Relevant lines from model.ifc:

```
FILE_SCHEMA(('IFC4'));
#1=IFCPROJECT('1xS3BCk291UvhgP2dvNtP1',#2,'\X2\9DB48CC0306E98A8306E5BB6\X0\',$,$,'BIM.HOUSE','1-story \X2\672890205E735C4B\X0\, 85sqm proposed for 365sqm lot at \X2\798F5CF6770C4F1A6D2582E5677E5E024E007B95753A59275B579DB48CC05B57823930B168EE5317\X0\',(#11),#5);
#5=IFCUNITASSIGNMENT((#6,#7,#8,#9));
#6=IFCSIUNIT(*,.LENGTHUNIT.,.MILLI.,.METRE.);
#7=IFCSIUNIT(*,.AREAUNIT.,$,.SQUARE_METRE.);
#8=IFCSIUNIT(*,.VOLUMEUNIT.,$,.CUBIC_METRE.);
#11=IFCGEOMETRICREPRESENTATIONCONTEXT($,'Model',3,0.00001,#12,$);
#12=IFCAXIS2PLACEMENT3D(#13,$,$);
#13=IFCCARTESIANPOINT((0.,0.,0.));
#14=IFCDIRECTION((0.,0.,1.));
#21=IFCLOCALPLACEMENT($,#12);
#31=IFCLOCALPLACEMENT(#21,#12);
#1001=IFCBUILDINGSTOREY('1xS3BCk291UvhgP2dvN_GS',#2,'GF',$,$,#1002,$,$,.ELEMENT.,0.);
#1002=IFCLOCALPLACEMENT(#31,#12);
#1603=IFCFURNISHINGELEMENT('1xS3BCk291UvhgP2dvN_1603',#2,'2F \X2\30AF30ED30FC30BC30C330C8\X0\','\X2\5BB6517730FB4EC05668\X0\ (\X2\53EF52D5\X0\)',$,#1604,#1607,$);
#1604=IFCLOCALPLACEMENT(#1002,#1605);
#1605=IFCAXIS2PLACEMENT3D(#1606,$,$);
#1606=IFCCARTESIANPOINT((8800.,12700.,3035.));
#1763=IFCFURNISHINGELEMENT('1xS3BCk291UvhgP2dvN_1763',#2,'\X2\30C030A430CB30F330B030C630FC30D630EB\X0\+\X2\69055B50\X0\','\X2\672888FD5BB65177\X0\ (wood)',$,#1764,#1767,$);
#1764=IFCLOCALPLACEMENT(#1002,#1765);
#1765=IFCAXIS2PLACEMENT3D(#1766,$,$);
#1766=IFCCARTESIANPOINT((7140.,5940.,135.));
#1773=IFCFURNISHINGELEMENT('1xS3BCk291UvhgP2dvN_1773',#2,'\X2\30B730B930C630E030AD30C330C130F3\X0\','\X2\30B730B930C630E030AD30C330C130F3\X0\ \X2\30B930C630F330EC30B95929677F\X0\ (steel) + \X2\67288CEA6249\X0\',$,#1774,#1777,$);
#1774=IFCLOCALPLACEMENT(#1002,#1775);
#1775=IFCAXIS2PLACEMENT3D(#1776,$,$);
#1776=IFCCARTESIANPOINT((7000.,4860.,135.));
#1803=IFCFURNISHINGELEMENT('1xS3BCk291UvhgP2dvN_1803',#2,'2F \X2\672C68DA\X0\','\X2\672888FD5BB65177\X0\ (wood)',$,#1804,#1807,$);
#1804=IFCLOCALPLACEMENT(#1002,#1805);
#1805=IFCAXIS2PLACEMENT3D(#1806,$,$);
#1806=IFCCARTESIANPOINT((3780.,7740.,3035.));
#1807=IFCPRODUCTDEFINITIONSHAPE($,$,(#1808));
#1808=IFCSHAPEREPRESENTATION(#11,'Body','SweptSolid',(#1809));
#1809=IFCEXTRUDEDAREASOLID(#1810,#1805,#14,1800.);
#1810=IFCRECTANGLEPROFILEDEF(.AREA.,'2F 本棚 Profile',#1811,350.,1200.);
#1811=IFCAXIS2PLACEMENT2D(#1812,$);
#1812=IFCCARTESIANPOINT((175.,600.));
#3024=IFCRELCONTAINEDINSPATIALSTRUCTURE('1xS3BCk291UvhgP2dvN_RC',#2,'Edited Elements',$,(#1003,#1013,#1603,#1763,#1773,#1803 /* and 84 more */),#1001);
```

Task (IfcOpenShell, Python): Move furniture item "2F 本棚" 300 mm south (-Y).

```python
import ifcopenshell
import ifcopenshell.api.geometry
import ifcopenshell.util.placement

model = ifcopenshell.open("model.ifc")

item = model.by_guid("1xS3BCk291UvhgP2dvN_1803")
matrix = ifcopenshell.util.placement.get_local_placement(item.ObjectPlacement)
matrix[1, 3] -= 300.0
ifcopenshell.api.geometry.edit_object_placement(model, product=item, matrix=matrix, is_si=False)

print(ifcopenshell.util.placement.get_local_placement(item.ObjectPlacement).round(3) + 0.0)

model.write("model-out.ifc")
```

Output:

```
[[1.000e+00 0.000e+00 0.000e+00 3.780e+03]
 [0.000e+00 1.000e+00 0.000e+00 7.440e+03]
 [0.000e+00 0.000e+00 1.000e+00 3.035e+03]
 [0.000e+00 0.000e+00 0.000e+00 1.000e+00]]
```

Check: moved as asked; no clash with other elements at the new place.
